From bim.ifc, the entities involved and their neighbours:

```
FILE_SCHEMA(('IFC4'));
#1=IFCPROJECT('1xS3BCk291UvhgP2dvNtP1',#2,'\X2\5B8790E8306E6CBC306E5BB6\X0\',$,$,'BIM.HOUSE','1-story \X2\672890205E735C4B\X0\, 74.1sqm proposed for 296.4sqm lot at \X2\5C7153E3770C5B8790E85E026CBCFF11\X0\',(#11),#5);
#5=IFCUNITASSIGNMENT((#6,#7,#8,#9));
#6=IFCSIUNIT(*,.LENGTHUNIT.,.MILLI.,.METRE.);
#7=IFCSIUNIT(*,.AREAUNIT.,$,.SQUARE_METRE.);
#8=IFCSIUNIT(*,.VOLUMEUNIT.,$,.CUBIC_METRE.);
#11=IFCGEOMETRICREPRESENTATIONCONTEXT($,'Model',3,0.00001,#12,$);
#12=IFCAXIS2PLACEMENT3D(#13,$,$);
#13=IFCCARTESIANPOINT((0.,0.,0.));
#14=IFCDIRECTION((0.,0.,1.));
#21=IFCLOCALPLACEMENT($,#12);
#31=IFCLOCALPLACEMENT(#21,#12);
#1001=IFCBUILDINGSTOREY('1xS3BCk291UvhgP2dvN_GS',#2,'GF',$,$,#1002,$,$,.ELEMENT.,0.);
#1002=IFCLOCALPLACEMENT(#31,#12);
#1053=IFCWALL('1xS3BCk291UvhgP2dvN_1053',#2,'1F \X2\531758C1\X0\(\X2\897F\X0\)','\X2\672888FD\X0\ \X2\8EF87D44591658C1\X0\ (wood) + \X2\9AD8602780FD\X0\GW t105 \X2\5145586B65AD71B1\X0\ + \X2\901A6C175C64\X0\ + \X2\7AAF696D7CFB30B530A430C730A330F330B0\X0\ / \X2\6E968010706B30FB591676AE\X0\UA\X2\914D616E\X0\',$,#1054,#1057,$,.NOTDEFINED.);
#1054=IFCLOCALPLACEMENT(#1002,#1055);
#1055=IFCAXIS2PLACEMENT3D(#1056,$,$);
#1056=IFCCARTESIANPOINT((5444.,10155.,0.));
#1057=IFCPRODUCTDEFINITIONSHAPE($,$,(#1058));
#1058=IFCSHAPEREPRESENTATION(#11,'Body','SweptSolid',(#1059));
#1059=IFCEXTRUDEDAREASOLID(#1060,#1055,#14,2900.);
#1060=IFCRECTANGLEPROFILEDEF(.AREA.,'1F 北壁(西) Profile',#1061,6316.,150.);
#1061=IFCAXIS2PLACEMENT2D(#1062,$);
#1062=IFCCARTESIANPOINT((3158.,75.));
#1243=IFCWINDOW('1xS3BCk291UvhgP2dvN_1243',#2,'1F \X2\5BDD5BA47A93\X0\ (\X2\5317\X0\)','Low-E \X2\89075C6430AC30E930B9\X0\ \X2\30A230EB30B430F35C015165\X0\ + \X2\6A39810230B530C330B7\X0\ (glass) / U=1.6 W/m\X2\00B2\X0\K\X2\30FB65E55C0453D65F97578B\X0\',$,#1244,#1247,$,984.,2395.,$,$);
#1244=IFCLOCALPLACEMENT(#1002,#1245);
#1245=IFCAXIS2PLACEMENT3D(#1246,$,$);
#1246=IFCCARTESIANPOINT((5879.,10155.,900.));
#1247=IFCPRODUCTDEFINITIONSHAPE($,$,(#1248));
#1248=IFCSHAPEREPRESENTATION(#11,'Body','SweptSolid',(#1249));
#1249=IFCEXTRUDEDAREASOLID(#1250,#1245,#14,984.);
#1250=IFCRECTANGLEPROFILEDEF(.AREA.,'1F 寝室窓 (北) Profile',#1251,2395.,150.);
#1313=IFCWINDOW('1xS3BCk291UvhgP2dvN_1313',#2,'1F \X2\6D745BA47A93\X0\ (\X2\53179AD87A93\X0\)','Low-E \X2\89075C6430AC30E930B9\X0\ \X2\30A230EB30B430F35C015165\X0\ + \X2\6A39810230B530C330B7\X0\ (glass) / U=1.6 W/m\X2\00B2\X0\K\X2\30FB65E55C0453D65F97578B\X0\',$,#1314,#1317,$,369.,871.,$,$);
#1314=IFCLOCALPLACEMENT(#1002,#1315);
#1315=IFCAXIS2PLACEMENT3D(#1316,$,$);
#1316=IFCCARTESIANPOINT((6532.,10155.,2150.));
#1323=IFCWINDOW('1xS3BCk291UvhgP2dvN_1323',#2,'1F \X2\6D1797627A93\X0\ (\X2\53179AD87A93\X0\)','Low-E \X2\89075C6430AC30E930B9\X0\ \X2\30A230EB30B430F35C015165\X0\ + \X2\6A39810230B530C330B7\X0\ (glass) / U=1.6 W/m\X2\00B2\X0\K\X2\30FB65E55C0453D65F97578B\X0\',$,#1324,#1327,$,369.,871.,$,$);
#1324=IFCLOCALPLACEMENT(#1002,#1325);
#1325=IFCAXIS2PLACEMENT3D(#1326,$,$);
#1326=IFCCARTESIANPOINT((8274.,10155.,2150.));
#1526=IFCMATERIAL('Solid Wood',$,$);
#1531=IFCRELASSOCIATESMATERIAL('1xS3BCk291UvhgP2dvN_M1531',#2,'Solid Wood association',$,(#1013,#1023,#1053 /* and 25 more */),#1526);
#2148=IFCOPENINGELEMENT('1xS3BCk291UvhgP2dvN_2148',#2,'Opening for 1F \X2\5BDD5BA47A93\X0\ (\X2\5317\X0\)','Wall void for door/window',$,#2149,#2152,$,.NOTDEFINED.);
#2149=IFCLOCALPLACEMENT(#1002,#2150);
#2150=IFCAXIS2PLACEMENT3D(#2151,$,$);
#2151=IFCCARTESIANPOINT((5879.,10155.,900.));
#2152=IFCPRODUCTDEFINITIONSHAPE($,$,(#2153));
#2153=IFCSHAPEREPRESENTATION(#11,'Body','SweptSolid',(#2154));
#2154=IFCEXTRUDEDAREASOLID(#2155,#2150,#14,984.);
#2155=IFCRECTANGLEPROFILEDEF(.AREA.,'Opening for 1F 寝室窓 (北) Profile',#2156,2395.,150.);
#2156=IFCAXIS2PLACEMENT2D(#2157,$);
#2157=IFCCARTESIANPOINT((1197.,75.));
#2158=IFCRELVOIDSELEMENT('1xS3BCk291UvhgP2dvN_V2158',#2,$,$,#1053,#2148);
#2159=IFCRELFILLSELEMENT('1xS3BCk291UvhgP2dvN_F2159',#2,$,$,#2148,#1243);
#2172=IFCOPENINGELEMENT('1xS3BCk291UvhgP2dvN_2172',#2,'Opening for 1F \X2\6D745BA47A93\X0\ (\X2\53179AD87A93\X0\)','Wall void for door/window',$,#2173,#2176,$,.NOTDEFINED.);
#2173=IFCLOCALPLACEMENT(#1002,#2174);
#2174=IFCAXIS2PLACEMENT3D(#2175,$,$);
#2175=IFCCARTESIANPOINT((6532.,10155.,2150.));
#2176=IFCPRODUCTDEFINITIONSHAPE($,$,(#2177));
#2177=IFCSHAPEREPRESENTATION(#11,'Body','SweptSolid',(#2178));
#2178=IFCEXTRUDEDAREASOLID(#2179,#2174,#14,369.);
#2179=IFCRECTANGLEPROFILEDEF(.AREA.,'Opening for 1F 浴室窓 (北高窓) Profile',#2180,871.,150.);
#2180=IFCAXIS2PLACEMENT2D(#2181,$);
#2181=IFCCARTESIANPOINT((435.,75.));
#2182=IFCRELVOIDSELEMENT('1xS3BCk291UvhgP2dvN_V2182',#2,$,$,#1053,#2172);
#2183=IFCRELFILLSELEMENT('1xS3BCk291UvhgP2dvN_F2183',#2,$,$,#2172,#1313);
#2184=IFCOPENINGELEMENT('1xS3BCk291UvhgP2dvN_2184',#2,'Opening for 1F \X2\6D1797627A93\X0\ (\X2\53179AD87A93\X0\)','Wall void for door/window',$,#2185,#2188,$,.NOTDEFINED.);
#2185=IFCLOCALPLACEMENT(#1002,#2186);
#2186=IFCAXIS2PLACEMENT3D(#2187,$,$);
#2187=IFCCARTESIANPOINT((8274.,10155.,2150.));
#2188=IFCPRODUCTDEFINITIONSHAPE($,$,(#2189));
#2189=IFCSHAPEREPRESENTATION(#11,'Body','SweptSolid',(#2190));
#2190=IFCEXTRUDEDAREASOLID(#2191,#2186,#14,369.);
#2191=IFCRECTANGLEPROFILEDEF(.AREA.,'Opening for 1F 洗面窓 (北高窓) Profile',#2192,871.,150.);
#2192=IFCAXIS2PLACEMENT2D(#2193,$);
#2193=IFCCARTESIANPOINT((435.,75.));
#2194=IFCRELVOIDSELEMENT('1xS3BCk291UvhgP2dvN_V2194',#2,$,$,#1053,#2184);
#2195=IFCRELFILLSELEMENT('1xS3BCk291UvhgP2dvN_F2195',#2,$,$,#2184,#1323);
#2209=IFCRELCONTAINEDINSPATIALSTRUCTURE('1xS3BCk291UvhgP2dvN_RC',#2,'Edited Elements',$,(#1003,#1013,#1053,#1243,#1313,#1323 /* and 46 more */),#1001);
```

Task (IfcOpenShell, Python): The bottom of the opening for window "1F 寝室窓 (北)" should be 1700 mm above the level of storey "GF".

```python
import numpy as np
import ifcopenshell
import ifcopenshell.api.geometry
import ifcopenshell.geom
import ifcopenshell.util.element
import ifcopenshell.util.placement
import ifcopenshell.util.shape
import ifcopenshell.util.unit

model = ifcopenshell.open("bim.ifc")
unit_scale = ifcopenshell.util.unit.calculate_unit_scale(model)

window = model.by_id(1243)
opening = window.FillsVoids[0].RelatingOpeningElement
storey = ifcopenshell.util.element.get_container(window, ifc_class="IfcBuildingStorey")
level = ifcopenshell.util.placement.get_local_placement(storey.ObjectPlacement)[2, 3]

# The opening's origin need not be at the sill, so measure its lowest point.
shape = ifcopenshell.geom.create_shape(ifcopenshell.geom.settings(), opening)
bottom = ifcopenshell.util.shape.get_shape_bottom_elevation(shape, shape.geometry) / unit_scale
dz = level + 1700.0 - bottom

shift = np.array([0.0, 0.0, dz])
# The window is not placed relative to its opening, so move both.
for product in (opening, window):
    matrix = ifcopenshell.util.placement.get_local_placement(product.ObjectPlacement)
    matrix[:3, 3] += shift
    ifcopenshell.api.geometry.edit_object_placement(model, product=product, matrix=matrix, is_si=False)

print(f"moved by {dz * unit_scale:+.3f} m")

model.write("bim-out.ifc")
```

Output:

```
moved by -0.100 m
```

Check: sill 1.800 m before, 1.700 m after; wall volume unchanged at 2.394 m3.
